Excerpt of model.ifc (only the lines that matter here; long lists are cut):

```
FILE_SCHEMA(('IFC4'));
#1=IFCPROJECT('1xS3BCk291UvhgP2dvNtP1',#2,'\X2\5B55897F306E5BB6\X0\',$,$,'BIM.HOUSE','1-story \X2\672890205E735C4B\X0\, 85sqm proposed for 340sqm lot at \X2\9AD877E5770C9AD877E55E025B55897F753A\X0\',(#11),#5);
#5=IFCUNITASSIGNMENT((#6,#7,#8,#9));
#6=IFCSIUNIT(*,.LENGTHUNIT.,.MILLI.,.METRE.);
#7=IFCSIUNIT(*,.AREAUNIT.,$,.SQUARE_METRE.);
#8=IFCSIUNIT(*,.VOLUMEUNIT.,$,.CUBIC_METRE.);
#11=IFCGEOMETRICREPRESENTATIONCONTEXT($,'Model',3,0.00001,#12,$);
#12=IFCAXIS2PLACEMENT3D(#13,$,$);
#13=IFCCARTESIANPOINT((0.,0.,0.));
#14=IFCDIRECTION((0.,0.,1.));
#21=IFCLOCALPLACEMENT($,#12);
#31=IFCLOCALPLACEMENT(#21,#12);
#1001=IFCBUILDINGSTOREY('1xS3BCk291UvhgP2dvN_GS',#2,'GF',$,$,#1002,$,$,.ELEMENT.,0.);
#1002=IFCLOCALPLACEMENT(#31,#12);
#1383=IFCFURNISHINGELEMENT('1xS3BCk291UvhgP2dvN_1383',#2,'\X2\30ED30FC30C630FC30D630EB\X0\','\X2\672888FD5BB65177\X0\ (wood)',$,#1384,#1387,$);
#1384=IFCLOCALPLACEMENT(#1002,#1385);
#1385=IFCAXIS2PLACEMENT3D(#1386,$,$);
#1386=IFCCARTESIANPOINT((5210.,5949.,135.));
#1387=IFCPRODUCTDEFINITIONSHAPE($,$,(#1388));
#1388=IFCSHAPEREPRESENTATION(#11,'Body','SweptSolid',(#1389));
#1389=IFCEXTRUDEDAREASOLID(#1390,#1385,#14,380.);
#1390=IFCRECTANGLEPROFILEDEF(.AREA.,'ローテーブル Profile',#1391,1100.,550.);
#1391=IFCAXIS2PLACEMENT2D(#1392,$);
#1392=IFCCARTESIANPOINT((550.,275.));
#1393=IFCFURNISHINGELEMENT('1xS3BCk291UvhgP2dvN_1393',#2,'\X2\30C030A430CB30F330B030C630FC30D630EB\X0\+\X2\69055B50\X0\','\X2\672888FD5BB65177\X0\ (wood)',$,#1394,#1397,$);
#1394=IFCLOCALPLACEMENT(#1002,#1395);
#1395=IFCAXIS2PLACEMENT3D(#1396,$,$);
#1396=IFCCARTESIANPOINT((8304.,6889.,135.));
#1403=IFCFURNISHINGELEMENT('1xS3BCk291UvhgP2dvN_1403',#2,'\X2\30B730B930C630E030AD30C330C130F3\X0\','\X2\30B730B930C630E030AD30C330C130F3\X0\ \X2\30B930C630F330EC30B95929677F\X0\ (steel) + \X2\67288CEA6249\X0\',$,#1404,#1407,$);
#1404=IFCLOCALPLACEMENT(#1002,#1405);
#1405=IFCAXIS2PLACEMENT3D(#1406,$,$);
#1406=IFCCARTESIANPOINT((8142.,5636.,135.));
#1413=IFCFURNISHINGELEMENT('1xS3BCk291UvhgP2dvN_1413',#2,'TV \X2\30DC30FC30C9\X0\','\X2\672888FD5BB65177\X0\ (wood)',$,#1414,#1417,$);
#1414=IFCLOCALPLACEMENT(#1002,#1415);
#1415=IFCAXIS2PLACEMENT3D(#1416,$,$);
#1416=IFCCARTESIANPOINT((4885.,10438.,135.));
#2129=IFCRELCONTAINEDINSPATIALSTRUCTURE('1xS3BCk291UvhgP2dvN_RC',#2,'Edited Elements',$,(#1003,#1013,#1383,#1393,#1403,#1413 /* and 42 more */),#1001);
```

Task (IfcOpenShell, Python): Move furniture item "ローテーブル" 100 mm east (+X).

```python
import ifcopenshell
import ifcopenshell.api.geometry
import ifcopenshell.util.placement
import ifcopenshell.util.unit

model = ifcopenshell.open("model.ifc")
unit_scale = ifcopenshell.util.unit.calculate_unit_scale(model)

item = model.by_guid("1xS3BCk291UvhgP2dvN_1383")
matrix = ifcopenshell.util.placement.get_local_placement(item.ObjectPlacement)
matrix[0, 3] += 0.1 / unit_scale
ifcopenshell.api.geometry.edit_object_placement(model, product=item, matrix=matrix, is_si=False)

print(ifcopenshell.util.placement.get_local_placement(item.ObjectPlacement).round(3) + 0.0)

model.write("model-out.ifc")
```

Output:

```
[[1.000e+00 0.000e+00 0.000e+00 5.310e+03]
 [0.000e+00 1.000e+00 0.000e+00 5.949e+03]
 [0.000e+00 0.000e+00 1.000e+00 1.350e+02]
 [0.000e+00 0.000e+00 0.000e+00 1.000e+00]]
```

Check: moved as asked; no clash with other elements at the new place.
